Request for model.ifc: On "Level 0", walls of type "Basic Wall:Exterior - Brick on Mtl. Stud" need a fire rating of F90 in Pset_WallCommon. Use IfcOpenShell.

First a look at what the model holds.

```python
import ifcopenshell
import ifcopenshell.util.element

model = ifcopenshell.open("model.ifc")
print(model.schema)
storey = next(s for s in model.by_type("IfcBuildingStorey") if s.Name == "Level 0")
walls = [e for e in ifcopenshell.util.element.get_decomposition(storey) if e.is_a("IfcWall")]
seen = {}
for e in walls:
    element_type = ifcopenshell.util.element.get_type(e)
    key = (element_type.Name if element_type != e and element_type else None, ifcopenshell.util.element.get_pset(e, "Pset_WallCommon", "FireRating"))
    seen[key] = seen.get(key, 0) + 1
for (name, value), count in sorted(seen.items(), key=str):
    print(count, "x", name, "|", value)
```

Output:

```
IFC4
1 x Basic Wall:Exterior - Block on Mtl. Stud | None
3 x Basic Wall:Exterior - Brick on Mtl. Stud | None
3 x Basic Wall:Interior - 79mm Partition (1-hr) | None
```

```python
import ifcopenshell
import ifcopenshell.api.pset
import ifcopenshell.util.element

model = ifcopenshell.open("model.ifc")

storey = next(s for s in model.by_type("IfcBuildingStorey") if s.Name == "Level 0")
walls = [e for e in ifcopenshell.util.element.get_decomposition(storey) if e.is_a("IfcWall")]

count = 0
for e in walls:
    element_type = ifcopenshell.util.element.get_type(e)
    if element_type in (None, e) or element_type.Name != "Basic Wall:Exterior - Brick on Mtl. Stud":
        continue
    # add_pset returns the element's existing set when there is one.
    pset = ifcopenshell.api.pset.add_pset(model, product=e, name="Pset_WallCommon")
    ifcopenshell.api.pset.edit_pset(model, pset=pset, properties={"FireRating": "F90"})
    count += 1

print(count, "walls updated")

model.write("model_v2.ifc")
```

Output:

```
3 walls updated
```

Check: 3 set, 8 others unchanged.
